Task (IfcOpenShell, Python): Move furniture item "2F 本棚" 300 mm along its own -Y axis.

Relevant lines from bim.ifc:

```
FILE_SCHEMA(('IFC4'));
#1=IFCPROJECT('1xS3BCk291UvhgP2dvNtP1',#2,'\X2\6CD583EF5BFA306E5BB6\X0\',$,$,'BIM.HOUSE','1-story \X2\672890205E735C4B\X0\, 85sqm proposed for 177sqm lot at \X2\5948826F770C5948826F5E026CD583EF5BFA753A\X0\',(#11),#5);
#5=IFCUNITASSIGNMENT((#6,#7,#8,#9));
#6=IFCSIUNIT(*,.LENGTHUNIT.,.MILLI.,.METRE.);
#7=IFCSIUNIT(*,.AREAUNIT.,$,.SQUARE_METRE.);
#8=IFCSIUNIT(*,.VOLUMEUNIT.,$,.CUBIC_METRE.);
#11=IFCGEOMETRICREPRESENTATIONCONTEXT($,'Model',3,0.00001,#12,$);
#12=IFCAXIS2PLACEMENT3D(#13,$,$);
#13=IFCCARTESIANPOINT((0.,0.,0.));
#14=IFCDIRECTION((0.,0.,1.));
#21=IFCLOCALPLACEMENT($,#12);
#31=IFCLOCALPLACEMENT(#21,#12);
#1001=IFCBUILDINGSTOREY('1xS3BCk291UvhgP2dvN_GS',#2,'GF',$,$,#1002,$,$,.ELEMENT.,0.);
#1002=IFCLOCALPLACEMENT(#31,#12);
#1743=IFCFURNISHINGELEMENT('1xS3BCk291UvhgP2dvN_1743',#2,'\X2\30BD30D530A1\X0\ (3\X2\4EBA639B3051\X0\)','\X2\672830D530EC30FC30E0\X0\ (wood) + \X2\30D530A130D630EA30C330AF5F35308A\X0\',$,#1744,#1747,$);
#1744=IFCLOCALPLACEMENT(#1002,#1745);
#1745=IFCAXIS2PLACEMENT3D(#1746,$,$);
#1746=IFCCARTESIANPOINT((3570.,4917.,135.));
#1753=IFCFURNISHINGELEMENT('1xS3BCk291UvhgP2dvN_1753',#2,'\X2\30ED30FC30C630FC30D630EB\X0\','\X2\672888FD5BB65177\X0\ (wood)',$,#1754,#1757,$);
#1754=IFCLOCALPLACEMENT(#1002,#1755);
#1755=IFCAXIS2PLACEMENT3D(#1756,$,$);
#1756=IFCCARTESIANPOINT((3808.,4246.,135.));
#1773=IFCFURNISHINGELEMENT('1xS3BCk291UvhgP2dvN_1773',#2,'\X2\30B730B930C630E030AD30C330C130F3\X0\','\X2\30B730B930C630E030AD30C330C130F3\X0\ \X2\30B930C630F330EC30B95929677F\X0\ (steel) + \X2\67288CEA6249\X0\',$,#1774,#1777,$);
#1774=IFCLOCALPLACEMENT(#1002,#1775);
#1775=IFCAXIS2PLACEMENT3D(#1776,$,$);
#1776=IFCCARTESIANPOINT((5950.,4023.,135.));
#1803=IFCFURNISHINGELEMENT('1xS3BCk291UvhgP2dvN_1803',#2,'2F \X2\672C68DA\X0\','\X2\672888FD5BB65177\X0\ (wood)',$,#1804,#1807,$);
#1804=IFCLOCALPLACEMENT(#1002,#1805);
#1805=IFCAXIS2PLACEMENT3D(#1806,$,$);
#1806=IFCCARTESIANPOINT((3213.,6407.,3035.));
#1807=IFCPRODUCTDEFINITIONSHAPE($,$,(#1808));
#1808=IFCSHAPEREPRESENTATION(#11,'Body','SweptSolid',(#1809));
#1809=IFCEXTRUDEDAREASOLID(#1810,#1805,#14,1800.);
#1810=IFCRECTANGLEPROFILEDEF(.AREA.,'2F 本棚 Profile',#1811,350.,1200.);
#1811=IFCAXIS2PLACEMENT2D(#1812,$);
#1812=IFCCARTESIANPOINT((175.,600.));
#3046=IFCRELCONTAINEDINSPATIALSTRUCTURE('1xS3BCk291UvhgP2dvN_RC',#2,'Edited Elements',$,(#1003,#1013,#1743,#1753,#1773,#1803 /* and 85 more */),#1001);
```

```python
import ifcopenshell
import ifcopenshell.api.geometry
import ifcopenshell.util.placement
import ifcopenshell.util.unit

model = ifcopenshell.open("bim.ifc")
unit_scale = ifcopenshell.util.unit.calculate_unit_scale(model)

item = model.by_guid("1xS3BCk291UvhgP2dvN_1803")
matrix = ifcopenshell.util.placement.get_local_placement(item.ObjectPlacement)
matrix[:3, 3] -= matrix[:3, 1] * 0.3 / unit_scale
ifcopenshell.api.geometry.edit_object_placement(model, product=item, matrix=matrix, is_si=False)

print(ifcopenshell.util.placement.get_local_placement(item.ObjectPlacement).round(3) + 0.0)

model.write("bim_v2.ifc")
```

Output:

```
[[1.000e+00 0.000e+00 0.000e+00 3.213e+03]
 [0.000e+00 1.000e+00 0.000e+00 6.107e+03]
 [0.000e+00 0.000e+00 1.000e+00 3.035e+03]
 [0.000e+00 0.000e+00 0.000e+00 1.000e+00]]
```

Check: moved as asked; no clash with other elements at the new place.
